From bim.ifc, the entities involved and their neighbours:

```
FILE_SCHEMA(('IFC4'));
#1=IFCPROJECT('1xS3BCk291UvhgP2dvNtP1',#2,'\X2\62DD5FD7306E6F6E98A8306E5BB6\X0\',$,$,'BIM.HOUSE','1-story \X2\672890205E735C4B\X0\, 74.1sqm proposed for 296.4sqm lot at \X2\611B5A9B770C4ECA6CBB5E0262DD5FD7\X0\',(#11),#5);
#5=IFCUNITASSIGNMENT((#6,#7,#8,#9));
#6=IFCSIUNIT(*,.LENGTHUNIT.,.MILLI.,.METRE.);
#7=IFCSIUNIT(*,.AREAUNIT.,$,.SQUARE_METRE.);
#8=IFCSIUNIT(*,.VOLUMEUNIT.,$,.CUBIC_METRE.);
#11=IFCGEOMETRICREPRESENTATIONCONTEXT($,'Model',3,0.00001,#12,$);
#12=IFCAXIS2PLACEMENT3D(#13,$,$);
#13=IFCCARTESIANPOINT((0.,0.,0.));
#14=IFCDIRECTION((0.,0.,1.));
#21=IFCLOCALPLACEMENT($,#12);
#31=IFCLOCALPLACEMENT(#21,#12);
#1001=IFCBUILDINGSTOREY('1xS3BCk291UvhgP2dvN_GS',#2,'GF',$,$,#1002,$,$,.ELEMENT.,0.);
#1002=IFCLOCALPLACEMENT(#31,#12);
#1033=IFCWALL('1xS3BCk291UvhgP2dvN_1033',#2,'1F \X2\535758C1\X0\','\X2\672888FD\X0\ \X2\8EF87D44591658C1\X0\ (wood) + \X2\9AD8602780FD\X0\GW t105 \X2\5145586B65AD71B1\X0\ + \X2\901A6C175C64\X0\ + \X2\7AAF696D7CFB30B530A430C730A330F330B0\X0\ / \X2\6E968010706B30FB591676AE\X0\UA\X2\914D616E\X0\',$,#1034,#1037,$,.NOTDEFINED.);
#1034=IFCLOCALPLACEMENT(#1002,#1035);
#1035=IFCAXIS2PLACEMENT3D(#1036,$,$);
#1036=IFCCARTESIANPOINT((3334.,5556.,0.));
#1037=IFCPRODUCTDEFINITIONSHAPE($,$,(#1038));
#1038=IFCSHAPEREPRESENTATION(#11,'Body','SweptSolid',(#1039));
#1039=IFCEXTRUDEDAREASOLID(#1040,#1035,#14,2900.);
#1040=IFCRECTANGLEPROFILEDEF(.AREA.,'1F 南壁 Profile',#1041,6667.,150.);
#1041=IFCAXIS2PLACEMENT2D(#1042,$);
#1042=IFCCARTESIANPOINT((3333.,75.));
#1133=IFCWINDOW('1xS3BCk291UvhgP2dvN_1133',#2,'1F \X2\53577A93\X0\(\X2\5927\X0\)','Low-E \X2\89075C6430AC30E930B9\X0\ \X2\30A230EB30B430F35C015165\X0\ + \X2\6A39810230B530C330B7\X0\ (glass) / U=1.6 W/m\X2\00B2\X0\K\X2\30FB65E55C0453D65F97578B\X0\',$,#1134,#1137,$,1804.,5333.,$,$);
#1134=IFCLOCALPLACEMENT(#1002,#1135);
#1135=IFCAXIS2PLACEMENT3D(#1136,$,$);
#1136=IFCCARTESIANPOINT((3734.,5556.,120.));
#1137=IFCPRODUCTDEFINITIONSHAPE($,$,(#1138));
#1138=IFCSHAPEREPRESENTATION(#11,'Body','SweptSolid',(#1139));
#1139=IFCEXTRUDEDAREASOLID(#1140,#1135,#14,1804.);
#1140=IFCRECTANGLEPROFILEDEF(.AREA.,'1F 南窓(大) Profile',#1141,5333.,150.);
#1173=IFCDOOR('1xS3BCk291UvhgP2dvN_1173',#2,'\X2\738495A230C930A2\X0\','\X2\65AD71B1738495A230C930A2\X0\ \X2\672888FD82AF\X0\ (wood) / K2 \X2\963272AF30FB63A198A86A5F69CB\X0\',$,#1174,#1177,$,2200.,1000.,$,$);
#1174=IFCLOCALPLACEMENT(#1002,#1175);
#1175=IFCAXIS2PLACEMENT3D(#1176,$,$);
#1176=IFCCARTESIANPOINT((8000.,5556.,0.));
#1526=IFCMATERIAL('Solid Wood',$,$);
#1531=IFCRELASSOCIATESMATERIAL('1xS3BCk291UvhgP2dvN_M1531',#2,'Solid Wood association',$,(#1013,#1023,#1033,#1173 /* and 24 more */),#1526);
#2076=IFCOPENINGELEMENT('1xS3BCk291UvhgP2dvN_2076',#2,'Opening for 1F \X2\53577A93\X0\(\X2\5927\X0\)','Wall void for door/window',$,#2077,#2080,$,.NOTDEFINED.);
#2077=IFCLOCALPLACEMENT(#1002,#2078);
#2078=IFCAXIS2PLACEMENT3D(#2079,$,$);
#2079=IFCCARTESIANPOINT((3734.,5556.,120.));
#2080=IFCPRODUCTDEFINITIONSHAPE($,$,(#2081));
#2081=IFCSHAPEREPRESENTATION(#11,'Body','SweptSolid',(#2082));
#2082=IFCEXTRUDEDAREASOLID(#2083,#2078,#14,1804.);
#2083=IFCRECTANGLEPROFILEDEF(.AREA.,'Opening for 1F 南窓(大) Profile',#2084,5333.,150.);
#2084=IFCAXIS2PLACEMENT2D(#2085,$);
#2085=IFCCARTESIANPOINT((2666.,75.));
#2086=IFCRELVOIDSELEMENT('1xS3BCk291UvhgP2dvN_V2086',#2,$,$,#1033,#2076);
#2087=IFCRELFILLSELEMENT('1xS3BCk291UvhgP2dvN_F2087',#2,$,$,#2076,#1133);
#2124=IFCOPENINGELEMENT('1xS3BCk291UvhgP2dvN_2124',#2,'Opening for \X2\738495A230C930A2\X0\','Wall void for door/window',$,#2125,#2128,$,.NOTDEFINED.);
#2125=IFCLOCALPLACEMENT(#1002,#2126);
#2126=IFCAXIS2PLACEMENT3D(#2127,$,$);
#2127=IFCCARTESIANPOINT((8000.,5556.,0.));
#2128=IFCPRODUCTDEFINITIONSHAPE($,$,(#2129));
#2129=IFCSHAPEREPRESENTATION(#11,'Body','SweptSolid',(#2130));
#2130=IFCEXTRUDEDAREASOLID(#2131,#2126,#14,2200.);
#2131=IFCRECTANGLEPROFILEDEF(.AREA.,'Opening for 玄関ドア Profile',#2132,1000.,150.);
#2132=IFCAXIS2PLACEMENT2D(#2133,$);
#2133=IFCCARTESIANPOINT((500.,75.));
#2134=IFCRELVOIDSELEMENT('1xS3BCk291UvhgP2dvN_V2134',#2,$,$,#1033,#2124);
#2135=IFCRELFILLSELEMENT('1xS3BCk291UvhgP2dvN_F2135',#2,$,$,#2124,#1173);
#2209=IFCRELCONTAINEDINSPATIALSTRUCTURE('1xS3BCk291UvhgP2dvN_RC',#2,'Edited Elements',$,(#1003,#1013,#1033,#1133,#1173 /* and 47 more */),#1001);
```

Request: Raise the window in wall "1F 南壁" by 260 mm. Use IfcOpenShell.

```python
import numpy as np
import ifcopenshell
import ifcopenshell.api.geometry
import ifcopenshell.util.placement
import ifcopenshell.util.unit

model = ifcopenshell.open("bim.ifc")
unit_scale = ifcopenshell.util.unit.calculate_unit_scale(model)

window = model.by_id(1133)
opening = window.FillsVoids[0].RelatingOpeningElement
dz = 260.0

shift = np.array([0.0, 0.0, dz])
# The window is not placed relative to its opening, so move both.
for product in (opening, window):
    matrix = ifcopenshell.util.placement.get_local_placement(product.ObjectPlacement)
    matrix[:3, 3] += shift
    ifcopenshell.api.geometry.edit_object_placement(model, product=product, matrix=matrix, is_si=False)

print(f"moved by {dz * unit_scale:+.3f} m")

model.write("bim_updated.ifc")
```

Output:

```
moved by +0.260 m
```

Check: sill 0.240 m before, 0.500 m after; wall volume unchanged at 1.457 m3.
